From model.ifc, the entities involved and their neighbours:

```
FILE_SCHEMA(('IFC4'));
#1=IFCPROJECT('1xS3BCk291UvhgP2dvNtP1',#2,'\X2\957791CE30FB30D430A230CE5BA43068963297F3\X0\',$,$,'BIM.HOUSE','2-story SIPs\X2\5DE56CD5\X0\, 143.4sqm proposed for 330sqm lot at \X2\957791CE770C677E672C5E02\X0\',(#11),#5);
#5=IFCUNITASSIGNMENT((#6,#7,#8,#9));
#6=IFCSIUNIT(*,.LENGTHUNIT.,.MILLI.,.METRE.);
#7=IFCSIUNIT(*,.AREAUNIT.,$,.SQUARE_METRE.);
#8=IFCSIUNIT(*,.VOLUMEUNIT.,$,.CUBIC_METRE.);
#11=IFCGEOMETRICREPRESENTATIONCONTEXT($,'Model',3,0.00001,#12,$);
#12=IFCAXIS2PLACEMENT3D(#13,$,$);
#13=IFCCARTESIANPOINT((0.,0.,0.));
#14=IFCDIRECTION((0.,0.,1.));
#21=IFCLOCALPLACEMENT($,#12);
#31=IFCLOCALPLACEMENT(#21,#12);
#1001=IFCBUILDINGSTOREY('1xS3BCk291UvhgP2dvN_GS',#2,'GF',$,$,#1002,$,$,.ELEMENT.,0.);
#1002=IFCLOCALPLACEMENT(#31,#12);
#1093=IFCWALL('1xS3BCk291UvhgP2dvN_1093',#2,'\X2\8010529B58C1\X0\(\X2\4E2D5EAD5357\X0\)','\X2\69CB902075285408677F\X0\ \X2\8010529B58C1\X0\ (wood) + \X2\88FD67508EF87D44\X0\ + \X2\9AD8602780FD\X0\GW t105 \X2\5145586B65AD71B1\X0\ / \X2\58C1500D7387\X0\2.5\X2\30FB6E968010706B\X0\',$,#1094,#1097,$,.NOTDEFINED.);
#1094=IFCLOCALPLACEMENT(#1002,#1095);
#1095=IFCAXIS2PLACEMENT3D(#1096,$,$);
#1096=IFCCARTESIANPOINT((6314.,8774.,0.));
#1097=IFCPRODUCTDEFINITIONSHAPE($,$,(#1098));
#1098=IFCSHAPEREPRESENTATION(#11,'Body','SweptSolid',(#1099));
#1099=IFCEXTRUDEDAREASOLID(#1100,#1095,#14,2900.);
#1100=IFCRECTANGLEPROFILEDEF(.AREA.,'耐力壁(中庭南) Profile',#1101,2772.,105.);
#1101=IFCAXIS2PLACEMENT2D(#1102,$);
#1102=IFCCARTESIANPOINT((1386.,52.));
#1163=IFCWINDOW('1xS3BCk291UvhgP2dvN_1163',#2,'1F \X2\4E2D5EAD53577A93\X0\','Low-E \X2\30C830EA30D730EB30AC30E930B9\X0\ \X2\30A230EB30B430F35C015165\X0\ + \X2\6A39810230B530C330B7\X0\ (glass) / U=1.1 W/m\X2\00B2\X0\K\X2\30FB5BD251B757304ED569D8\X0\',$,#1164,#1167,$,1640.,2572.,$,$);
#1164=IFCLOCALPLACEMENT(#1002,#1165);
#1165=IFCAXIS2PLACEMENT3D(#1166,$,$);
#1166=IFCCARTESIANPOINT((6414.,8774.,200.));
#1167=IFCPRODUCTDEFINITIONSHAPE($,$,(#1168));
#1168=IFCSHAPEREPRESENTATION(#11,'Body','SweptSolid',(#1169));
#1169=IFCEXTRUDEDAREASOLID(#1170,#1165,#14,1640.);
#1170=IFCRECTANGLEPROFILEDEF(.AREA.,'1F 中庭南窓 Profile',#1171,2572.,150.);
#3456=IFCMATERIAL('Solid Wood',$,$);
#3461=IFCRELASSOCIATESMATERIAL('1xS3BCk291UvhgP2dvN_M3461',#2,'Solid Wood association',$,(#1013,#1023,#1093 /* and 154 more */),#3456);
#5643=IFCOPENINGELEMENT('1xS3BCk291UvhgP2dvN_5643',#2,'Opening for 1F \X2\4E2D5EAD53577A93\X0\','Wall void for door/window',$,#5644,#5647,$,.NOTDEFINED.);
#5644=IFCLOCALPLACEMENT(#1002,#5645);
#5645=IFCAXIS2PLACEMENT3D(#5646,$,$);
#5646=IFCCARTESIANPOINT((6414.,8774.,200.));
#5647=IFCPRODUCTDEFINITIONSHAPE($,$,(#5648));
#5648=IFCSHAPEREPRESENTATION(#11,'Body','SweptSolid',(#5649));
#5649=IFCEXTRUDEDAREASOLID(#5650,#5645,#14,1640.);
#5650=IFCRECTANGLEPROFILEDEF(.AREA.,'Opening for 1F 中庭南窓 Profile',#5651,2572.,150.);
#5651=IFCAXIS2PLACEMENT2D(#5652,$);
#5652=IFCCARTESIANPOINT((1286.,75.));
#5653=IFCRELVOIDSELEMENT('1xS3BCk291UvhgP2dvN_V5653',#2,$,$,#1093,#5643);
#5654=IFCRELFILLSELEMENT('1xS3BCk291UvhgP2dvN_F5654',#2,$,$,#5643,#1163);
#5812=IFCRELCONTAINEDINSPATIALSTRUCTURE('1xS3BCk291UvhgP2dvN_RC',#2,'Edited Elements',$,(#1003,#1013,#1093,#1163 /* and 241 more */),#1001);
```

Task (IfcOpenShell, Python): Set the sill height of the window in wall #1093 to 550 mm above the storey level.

```python
import numpy as np
import ifcopenshell
import ifcopenshell.api.geometry
import ifcopenshell.geom
import ifcopenshell.util.element
import ifcopenshell.util.placement
import ifcopenshell.util.shape
import ifcopenshell.util.unit

model = ifcopenshell.open("model.ifc")
unit_scale = ifcopenshell.util.unit.calculate_unit_scale(model)

window = model.by_id(1163)
opening = window.FillsVoids[0].RelatingOpeningElement
storey = ifcopenshell.util.element.get_container(window, ifc_class="IfcBuildingStorey")
level = ifcopenshell.util.placement.get_local_placement(storey.ObjectPlacement)[2, 3]

# The opening's origin need not be at the sill, so measure its lowest point.
shape = ifcopenshell.geom.create_shape(ifcopenshell.geom.settings(), opening)
bottom = ifcopenshell.util.shape.get_shape_bottom_elevation(shape, shape.geometry) / unit_scale
dz = level + 550.0 - bottom

shift = np.array([0.0, 0.0, dz])
# The window is not placed relative to its opening, so move both.
for product in (opening, window):
    matrix = ifcopenshell.util.placement.get_local_placement(product.ObjectPlacement)
    matrix[:3, 3] += shift
    ifcopenshell.api.geometry.edit_object_placement(model, product=product, matrix=matrix, is_si=False)

print(f"moved by {dz * unit_scale:+.3f} m")

model.write("model-out.ifc")
```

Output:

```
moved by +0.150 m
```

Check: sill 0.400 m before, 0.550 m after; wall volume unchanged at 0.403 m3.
